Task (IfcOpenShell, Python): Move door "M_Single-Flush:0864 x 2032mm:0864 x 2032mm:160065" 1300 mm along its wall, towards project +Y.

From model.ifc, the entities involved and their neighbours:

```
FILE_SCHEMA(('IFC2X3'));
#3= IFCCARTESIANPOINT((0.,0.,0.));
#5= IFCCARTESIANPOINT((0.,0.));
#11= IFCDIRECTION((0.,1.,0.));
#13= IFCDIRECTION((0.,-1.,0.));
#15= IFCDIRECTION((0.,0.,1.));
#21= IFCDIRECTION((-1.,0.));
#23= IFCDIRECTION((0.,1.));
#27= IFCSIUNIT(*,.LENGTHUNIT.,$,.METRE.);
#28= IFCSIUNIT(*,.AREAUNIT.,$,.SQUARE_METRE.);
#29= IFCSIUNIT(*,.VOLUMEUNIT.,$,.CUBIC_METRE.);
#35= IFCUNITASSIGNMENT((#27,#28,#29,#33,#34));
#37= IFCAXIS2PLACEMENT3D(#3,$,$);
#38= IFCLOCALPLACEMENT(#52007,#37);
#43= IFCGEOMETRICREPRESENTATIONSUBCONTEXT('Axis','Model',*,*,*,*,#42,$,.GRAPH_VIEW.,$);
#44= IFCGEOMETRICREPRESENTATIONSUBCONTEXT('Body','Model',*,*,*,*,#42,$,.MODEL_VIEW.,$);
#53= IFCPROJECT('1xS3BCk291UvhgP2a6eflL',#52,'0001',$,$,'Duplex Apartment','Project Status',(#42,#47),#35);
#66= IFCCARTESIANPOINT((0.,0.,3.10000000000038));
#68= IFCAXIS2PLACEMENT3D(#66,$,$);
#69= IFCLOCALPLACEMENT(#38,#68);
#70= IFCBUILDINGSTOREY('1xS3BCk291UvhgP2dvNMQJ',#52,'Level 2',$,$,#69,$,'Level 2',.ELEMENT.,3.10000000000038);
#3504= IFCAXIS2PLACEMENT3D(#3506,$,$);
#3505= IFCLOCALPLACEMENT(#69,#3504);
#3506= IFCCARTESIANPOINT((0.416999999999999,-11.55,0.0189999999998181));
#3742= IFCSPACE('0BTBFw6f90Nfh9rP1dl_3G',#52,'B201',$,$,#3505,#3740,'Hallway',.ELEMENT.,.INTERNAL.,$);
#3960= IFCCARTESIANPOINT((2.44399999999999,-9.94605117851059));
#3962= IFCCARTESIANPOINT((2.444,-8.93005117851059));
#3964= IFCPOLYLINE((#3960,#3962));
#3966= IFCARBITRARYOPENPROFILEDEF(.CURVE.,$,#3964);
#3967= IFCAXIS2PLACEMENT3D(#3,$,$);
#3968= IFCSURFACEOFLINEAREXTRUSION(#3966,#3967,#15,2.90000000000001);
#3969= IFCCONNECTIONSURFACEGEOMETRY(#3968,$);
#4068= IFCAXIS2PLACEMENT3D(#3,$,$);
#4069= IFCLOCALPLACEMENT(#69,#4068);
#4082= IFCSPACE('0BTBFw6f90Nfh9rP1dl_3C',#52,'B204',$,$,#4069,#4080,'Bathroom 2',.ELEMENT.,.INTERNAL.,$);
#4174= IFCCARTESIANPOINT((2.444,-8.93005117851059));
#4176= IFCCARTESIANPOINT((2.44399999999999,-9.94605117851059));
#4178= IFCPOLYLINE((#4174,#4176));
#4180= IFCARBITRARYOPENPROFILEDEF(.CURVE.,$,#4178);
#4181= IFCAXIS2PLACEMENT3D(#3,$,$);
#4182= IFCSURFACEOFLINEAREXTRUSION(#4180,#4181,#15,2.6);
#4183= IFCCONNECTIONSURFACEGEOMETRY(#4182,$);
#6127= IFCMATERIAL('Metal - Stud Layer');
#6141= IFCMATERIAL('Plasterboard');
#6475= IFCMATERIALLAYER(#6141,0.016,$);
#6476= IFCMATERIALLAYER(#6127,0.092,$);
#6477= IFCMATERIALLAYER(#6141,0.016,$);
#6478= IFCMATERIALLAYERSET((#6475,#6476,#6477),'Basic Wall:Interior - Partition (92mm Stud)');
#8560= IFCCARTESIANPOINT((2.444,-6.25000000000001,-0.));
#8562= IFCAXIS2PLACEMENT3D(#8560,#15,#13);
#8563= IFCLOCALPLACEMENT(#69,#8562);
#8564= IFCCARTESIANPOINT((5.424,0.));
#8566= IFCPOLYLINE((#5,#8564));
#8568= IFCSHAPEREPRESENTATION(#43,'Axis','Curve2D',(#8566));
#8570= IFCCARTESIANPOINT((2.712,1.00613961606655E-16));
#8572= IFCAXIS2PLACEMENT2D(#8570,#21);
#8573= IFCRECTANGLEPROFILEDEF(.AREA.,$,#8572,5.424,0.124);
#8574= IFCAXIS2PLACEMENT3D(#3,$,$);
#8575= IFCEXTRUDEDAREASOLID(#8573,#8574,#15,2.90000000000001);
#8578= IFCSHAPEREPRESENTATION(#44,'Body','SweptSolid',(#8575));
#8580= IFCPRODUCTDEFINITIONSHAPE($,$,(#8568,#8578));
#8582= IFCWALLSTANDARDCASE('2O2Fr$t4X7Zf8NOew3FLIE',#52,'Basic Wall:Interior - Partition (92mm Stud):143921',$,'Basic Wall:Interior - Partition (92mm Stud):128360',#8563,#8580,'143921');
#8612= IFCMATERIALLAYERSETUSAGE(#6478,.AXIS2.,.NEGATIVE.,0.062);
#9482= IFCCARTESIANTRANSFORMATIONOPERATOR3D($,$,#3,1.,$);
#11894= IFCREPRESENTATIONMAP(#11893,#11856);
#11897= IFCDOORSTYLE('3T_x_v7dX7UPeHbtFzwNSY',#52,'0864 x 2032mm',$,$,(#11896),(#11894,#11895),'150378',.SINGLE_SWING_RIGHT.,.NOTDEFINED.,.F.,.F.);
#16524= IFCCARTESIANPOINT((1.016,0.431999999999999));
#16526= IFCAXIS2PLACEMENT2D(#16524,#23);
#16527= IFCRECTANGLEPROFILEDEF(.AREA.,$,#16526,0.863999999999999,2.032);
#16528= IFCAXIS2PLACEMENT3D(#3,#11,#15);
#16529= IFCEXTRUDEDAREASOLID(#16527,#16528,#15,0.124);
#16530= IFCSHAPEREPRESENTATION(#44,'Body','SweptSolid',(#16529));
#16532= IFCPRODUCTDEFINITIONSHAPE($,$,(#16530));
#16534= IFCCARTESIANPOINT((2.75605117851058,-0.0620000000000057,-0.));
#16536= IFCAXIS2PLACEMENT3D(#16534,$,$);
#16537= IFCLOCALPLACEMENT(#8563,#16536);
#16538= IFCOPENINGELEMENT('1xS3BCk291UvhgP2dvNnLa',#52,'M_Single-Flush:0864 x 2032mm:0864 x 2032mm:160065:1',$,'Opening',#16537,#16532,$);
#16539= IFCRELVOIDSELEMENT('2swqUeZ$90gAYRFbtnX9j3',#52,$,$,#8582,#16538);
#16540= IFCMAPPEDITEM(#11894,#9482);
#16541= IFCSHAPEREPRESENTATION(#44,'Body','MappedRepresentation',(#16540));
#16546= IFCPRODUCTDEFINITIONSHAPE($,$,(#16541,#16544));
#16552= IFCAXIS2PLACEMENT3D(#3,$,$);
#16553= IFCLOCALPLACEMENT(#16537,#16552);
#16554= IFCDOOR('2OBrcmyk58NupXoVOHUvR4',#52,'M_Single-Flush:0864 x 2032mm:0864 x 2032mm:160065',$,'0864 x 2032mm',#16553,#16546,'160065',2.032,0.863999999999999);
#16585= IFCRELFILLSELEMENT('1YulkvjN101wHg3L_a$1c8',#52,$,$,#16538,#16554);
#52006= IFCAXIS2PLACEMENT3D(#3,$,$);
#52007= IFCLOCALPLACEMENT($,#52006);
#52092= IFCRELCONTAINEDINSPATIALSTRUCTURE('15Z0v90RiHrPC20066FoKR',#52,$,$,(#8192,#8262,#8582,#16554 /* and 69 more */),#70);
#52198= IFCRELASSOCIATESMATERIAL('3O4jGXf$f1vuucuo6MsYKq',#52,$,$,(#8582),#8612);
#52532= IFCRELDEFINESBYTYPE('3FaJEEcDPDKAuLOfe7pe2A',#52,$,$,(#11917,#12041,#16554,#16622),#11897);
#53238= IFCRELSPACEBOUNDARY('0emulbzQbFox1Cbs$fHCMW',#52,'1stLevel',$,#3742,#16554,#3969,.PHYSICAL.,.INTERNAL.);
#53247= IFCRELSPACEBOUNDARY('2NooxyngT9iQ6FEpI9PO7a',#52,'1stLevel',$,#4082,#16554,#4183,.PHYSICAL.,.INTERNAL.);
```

```python
import numpy as np
import ifcopenshell
import ifcopenshell.api.geometry
import ifcopenshell.util.placement
import ifcopenshell.util.unit

model = ifcopenshell.open("model.ifc")
unit_scale = ifcopenshell.util.unit.calculate_unit_scale(model)

door = model.by_id(16554)
opening = door.FillsVoids[0].RelatingOpeningElement
wall = opening.VoidsElements[0].RelatingBuildingElement

wall_matrix = ifcopenshell.util.placement.get_local_placement(wall.ObjectPlacement)
shift = wall_matrix[:3, 0] * -1.3 / unit_scale
before = ifcopenshell.util.placement.get_local_placement(door.ObjectPlacement)[:3, 3].copy()

# The door is placed relative to its opening, so it follows when the opening moves.
matrix = ifcopenshell.util.placement.get_local_placement(opening.ObjectPlacement)
matrix[:3, 3] += shift
ifcopenshell.api.geometry.edit_object_placement(
    model, product=opening, matrix=matrix, is_si=False, should_transform_children=True
)

# Space boundary surfaces are stored in each space's coordinates; move them too.
for rel in door.ProvidesBoundaries:
    if not rel.ConnectionGeometry:
        continue
    surface = rel.ConnectionGeometry.SurfaceOnRelatingElement
    space_matrix = ifcopenshell.util.placement.get_local_placement(rel.RelatingSpace.ObjectPlacement)
    point = np.array(surface.Position.Location.Coordinates) + space_matrix[:3, :3].T @ shift
    surface.Position = model.createIfcAxis2Placement3D(
        model.createIfcCartesianPoint(point.tolist()), surface.Position.Axis, surface.Position.RefDirection
    )

after = ifcopenshell.util.placement.get_local_placement(door.ObjectPlacement)[:3, 3]
print("door moved by", (after - before).round(3) + 0.0)

model.write("model_v2.ifc")
```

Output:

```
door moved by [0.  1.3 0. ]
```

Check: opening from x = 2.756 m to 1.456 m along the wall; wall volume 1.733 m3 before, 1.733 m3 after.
